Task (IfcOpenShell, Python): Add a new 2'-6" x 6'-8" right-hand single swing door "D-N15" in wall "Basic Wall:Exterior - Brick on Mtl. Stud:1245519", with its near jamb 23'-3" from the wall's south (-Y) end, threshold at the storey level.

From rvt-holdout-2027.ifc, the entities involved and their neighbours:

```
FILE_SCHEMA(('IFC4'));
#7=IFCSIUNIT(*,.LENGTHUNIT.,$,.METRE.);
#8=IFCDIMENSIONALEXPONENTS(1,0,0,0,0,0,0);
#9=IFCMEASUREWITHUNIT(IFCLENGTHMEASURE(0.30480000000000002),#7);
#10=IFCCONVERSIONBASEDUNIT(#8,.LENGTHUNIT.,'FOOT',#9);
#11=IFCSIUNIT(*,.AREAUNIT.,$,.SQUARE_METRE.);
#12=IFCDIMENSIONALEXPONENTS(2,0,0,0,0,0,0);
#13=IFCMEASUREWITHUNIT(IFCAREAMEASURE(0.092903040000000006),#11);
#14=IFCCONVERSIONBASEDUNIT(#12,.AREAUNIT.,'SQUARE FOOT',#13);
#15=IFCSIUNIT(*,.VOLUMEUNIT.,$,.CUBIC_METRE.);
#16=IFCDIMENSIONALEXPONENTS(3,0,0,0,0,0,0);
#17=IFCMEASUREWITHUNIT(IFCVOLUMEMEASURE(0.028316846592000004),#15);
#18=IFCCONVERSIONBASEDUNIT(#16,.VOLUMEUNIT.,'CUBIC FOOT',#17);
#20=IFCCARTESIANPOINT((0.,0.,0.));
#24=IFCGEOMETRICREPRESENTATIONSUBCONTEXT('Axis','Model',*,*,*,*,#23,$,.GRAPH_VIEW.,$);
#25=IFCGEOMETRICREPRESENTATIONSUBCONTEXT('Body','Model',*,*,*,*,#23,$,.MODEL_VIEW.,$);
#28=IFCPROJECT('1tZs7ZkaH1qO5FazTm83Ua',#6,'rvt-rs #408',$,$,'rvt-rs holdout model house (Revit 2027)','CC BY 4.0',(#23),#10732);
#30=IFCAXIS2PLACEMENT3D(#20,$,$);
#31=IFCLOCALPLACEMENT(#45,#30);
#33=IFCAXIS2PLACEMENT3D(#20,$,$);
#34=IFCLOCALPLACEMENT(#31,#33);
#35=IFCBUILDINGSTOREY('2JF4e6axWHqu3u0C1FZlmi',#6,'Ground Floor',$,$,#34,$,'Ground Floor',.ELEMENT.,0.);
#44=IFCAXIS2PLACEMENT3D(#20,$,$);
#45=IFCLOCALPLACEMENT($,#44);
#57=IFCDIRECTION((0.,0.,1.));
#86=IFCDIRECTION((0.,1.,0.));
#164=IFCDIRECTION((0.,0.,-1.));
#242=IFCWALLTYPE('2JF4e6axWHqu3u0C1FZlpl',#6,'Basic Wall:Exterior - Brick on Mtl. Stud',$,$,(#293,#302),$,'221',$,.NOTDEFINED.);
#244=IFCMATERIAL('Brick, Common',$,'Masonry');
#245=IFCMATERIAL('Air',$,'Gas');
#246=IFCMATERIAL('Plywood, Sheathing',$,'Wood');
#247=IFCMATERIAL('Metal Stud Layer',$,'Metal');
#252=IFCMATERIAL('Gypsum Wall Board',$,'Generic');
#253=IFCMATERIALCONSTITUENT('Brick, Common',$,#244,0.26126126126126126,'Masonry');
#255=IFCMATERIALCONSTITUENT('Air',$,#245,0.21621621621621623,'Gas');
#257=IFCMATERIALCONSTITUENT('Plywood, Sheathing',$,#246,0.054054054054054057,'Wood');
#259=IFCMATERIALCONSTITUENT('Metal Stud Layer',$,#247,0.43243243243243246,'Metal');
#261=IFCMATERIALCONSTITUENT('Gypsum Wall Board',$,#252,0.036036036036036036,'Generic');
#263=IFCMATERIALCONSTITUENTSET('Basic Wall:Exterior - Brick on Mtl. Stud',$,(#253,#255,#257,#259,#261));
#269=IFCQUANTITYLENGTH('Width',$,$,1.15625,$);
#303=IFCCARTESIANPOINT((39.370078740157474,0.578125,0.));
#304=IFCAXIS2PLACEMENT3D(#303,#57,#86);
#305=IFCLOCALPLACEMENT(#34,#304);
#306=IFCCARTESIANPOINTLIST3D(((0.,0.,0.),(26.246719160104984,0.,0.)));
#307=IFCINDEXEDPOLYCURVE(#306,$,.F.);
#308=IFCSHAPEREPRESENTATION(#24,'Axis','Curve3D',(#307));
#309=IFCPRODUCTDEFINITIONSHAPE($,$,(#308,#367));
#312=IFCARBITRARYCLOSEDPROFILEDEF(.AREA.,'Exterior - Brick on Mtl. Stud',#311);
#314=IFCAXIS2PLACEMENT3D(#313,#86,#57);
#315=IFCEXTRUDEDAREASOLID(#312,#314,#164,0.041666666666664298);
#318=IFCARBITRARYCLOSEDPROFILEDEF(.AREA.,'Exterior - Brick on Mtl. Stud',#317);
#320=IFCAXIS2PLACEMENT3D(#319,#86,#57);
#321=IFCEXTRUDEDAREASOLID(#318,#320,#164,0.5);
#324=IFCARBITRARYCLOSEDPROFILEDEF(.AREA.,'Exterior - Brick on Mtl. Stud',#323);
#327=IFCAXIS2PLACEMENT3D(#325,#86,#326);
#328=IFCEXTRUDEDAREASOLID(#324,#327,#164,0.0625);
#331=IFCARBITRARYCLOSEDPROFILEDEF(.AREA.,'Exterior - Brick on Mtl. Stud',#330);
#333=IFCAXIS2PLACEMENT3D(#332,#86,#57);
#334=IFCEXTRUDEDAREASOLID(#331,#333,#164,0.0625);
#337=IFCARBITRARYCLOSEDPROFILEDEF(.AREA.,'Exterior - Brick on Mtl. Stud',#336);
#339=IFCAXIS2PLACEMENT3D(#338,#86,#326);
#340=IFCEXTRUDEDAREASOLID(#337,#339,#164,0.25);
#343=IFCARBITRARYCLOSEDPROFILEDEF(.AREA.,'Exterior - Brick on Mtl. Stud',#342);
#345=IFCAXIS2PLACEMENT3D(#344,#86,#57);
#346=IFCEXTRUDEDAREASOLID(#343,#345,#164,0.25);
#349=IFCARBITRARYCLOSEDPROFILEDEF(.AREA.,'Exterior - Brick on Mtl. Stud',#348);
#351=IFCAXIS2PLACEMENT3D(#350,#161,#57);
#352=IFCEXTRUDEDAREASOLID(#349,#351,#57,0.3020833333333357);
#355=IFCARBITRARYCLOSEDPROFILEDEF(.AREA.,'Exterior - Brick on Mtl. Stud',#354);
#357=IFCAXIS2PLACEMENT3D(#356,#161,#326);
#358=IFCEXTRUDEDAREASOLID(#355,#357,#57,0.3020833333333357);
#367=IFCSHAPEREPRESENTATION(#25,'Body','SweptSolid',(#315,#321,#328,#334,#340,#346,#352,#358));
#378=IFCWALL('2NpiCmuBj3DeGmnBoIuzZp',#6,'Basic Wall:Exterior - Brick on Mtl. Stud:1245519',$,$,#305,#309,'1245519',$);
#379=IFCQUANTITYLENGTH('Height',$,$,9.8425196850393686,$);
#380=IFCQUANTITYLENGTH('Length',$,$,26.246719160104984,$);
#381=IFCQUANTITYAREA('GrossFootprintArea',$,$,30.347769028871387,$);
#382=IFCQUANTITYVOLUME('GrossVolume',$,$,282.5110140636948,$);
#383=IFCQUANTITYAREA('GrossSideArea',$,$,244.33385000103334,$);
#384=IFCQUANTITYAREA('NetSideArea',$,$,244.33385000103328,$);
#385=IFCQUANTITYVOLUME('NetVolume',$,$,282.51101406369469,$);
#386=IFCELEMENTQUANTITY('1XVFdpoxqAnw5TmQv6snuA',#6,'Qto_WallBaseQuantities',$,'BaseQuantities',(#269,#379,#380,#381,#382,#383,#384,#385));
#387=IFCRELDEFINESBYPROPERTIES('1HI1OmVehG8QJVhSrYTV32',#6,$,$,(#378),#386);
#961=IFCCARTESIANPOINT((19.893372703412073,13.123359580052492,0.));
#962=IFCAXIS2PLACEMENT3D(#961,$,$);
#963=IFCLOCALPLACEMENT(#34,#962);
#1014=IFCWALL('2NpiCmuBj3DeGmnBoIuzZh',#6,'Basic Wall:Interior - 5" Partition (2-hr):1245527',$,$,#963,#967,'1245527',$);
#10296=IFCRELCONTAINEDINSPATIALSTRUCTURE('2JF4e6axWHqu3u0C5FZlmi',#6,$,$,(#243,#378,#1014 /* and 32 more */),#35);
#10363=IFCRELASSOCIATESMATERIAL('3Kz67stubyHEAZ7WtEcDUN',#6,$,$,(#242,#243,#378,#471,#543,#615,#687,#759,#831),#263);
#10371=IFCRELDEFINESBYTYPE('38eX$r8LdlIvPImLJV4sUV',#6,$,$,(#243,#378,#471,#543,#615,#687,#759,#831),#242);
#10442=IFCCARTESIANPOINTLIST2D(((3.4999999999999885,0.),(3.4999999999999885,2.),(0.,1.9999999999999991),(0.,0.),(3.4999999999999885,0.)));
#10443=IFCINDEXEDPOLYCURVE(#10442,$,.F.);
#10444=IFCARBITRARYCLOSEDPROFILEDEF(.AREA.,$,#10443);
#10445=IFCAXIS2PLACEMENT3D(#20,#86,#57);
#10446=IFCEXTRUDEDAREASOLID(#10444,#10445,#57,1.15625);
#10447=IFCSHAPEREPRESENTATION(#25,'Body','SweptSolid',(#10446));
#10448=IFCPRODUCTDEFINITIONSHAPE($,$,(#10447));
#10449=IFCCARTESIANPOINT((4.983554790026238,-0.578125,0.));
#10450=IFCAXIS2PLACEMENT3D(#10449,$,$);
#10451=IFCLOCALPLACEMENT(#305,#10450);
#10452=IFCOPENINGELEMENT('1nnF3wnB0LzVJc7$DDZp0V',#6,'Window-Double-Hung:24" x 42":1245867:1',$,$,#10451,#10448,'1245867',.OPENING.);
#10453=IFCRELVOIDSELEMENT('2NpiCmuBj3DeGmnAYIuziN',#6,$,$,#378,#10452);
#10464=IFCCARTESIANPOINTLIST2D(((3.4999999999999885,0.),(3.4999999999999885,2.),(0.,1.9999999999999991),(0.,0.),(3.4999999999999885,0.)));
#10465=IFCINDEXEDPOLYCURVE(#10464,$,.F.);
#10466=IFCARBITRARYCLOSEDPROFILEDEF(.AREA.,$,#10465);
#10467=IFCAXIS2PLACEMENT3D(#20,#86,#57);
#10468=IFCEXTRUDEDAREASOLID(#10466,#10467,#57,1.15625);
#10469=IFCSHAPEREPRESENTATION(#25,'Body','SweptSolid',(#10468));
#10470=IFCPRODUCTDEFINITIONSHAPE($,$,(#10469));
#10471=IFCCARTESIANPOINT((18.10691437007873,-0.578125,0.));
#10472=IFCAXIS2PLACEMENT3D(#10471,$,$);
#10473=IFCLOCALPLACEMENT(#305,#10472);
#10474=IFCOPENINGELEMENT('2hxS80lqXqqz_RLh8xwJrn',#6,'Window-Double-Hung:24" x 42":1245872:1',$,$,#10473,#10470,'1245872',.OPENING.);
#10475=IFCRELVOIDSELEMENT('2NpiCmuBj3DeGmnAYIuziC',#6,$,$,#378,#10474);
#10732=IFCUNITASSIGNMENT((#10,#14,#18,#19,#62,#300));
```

```python
import numpy as np
import ifcopenshell
import ifcopenshell.api.feature
import ifcopenshell.api.geometry
import ifcopenshell.api.pset
import ifcopenshell.api.root
import ifcopenshell.api.spatial
import ifcopenshell.geom
import ifcopenshell.util.element
import ifcopenshell.util.placement
import ifcopenshell.util.representation
import ifcopenshell.util.shape
import ifcopenshell.util.unit

model = ifcopenshell.open("rvt-holdout-2027.ifc")
unit_scale = ifcopenshell.util.unit.calculate_unit_scale(model)
area_scale = ifcopenshell.util.unit.calculate_unit_scale(model, "AREAUNIT")
volume_scale = ifcopenshell.util.unit.calculate_unit_scale(model, "VOLUMEUNIT")
settings = ifcopenshell.geom.settings()


def volume(element):
    """Net volume in cubic metres, openings subtracted."""
    shape = ifcopenshell.geom.create_shape(settings, element)
    return ifcopenshell.util.shape.get_volume(shape.geometry)


wall = model.by_guid("2NpiCmuBj3DeGmnBoIuzZp")
storey = ifcopenshell.util.element.get_container(wall, ifc_class="IfcBuildingStorey")
context = ifcopenshell.util.representation.get_context(model, "Model", "Body", "MODEL_VIEW")
before = volume(wall)

width, height, from_end, sill = 0.762, 2.032, 7.0866, 0.0  # metres

# The wall runs along its own X axis, and the end named is its -X end.
wall_shape = ifcopenshell.geom.create_shape(settings, wall)
x, y, z = ifcopenshell.util.shape.get_vertices(wall_shape.geometry).T
start = x.min() + from_end
face, thickness = float(y.min()), float(y.max() - y.min())
wall_matrix = ifcopenshell.util.placement.get_local_placement(wall.ObjectPlacement)
level = ifcopenshell.util.placement.get_local_placement(storey.ObjectPlacement)[2, 3]


def in_wall(x, y):
    """Placement at x, y metres in the wall's axes, at sill height."""
    matrix = wall_matrix.copy()
    matrix[:, 3] = wall_matrix @ np.array([x / unit_scale, y / unit_scale, 0.0, 1.0])
    matrix[2, 3] = level + sill / unit_scale
    return matrix


# Opening: a box that overshoots both wall faces by 50 mm.
opening = ifcopenshell.api.root.create_entity(model, ifc_class="IfcOpeningElement", predefined_type="OPENING")
box = ifcopenshell.api.geometry.add_wall_representation(
    model, context=context, length=width, height=height, thickness=thickness + 0.1
)
ifcopenshell.api.geometry.assign_representation(model, product=opening, representation=box)
ifcopenshell.api.geometry.edit_object_placement(model, product=opening, matrix=in_wall(start, face - 0.05), is_si=False)
ifcopenshell.api.feature.add_feature(model, feature=opening, element=wall)

door = ifcopenshell.api.root.create_entity(model, ifc_class="IfcDoor", name="D-N15", predefined_type="DOOR")
door.OverallWidth, door.OverallHeight = width / unit_scale, height / unit_scale
door.OperationType = "SINGLE_SWING_RIGHT"
body = ifcopenshell.api.geometry.add_door_representation(
    model,
    context=context,
    overall_width=door.OverallWidth,
    overall_height=door.OverallHeight,
    operation_type="SINGLE_SWING_RIGHT",
    lining_properties={"LiningDepth": thickness / unit_scale, "ThresholdDepth": thickness / unit_scale},
)
ifcopenshell.api.geometry.assign_representation(model, product=door, representation=body)
ifcopenshell.api.spatial.assign_container(model, products=[door], relating_structure=storey)
ifcopenshell.api.feature.add_filling(model, opening=opening, element=door)

# The lining spans the wall, so the door starts at the wall face.
ifcopenshell.api.geometry.edit_object_placement(model, product=door, matrix=in_wall(start, face), is_si=False)

after = volume(wall)

# Update the wall's stored quantities.
qto = model.by_id(ifcopenshell.util.element.get_pset(wall, "Qto_WallBaseQuantities", should_inherit=False)["id"])
ifcopenshell.api.pset.edit_qto(model, qto=qto, properties={
    "NetSideArea": after / thickness / area_scale,
    "NetVolume": after / volume_scale,
})

print(f"wall volume {before:.3f} -> {after:.3f} m3")

model.write("rvt-holdout-2027_updated.ifc")
```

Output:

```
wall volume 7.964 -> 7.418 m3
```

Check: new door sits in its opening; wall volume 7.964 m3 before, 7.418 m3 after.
